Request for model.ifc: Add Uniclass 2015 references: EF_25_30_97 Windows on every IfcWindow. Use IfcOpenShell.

First a look at what the model holds.

```python
import ifcopenshell

model = ifcopenshell.open("model.ifc")
print(model.schema)
print("classifications:", [c.Name for c in model.by_type("IfcClassification")])
for ifc_class in ("IfcDoor", "IfcRoof", "IfcStair", "IfcWall", "IfcWindow"):
    print(ifc_class, len(model.by_type(ifc_class)))
```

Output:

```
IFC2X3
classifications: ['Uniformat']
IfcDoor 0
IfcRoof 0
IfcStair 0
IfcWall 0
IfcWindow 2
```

```python
import ifcopenshell
import ifcopenshell.api.classification

model = ifcopenshell.open("model.ifc")

# IFC2X3 requires Source and Edition and has no link from the project to the system.
system = model.create_entity("IfcClassification", Source="NBS", Edition="2015", Name="Uniclass 2015")

codes = {
    "IfcWindow": ("EF_25_30_97", "Windows"),
}
for ifc_class, (code, name) in codes.items():
    products = model.by_type(ifc_class)
    ifcopenshell.api.classification.add_reference(
        model, products=products, classification=system, identification=code, name=name
    )
    print(code, len(products))

model.write("model-out.ifc")
```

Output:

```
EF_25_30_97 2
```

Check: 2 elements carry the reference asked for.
